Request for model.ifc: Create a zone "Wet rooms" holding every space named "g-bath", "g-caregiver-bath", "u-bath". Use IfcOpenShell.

First a look at what the model holds.

```python
import ifcopenshell

model = ifcopenshell.open("model.ifc")
print(model.schema)
seen = {}
for space in model.by_type("IfcSpace"):
    seen[space.LongName] = seen.get(space.LongName, 0) + 1
for name, count in sorted(seen.items(), key=str):
    print(count, "x", name)
print("zones:", [z.Name for z in model.by_type("IfcZone")][:20])
```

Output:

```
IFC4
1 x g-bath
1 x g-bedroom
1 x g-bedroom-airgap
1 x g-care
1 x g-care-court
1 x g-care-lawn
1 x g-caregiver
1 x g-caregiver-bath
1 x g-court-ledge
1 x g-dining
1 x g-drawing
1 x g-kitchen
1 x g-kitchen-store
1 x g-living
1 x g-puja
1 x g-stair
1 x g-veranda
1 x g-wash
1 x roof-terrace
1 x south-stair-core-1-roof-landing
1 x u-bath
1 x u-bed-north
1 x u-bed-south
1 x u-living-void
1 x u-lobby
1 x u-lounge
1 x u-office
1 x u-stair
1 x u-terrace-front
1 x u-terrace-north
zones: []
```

```python
import ifcopenshell
import ifcopenshell.api.group
import ifcopenshell.api.root

model = ifcopenshell.open("model.ifc")

names = {"g-bath", "g-caregiver-bath", "u-bath"}
spaces = [s for s in model.by_type("IfcSpace") if s.LongName in names]

zone = ifcopenshell.api.root.create_entity(model, ifc_class="IfcZone", name="Wet rooms")
ifcopenshell.api.group.assign_group(model, products=spaces, group=zone)
print(len(spaces), "spaces in", zone.Name)

model.write("model_rev.ifc")
```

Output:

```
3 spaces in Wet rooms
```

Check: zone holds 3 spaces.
